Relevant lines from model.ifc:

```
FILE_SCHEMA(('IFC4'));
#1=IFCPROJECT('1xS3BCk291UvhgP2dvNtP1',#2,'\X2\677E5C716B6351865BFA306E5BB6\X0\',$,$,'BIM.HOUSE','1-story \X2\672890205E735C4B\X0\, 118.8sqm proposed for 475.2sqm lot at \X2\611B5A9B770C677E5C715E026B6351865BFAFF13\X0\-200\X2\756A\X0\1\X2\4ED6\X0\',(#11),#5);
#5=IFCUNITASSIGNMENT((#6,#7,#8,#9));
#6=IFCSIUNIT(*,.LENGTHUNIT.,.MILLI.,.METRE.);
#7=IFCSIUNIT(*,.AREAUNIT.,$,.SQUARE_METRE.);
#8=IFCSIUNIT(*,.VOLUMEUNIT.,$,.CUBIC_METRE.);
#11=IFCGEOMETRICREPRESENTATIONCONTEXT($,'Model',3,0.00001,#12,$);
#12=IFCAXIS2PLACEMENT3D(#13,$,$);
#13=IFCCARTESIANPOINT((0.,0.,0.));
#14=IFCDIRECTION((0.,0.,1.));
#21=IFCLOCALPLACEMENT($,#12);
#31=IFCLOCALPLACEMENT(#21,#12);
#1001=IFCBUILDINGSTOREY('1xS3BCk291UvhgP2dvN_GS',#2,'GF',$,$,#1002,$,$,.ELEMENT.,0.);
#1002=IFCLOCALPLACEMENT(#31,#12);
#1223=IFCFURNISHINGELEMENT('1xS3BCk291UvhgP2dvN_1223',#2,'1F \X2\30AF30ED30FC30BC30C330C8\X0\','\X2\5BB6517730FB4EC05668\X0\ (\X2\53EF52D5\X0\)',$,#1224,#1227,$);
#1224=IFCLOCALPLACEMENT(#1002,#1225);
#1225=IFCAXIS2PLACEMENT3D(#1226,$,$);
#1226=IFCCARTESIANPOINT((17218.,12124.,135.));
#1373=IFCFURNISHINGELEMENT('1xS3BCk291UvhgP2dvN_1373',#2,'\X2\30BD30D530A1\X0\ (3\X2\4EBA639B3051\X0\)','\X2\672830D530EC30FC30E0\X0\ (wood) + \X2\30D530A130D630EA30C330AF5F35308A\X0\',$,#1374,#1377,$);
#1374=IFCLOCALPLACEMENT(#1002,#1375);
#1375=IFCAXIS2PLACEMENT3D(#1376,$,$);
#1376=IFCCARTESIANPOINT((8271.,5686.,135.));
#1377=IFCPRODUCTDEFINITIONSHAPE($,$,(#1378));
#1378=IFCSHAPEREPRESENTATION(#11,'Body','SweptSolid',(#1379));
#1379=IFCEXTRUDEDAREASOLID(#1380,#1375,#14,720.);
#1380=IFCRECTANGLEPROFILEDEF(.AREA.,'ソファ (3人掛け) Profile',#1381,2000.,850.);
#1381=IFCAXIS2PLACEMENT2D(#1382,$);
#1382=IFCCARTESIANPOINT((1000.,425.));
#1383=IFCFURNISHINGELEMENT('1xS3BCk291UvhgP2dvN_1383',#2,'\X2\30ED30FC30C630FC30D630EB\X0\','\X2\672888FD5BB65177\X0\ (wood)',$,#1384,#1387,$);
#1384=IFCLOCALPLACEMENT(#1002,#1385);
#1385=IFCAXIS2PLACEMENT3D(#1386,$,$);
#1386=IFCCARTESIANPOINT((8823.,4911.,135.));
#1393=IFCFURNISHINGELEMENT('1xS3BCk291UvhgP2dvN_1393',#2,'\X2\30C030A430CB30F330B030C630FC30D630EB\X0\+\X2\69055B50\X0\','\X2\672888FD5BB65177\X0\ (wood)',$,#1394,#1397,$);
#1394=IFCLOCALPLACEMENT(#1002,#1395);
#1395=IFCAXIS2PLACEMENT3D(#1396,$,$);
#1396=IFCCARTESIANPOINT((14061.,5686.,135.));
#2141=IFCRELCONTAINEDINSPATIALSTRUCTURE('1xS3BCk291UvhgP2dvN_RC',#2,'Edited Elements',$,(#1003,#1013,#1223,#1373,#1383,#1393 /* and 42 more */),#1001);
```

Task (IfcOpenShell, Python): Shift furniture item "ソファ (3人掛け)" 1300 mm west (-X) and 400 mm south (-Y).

```python
import ifcopenshell
import ifcopenshell.api.geometry
import ifcopenshell.util.placement

model = ifcopenshell.open("model.ifc")

item = model.by_id(1373)
matrix = ifcopenshell.util.placement.get_local_placement(item.ObjectPlacement)
matrix[0, 3] -= 1300.0
matrix[1, 3] -= 400.0
ifcopenshell.api.geometry.edit_object_placement(model, product=item, matrix=matrix, is_si=False)

print(ifcopenshell.util.placement.get_local_placement(item.ObjectPlacement).round(3) + 0.0)

model.write("model_updated.ifc")
```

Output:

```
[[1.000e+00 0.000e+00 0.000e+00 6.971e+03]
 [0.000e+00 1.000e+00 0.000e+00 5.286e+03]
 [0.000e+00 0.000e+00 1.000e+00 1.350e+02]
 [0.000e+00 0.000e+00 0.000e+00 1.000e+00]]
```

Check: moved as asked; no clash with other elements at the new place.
